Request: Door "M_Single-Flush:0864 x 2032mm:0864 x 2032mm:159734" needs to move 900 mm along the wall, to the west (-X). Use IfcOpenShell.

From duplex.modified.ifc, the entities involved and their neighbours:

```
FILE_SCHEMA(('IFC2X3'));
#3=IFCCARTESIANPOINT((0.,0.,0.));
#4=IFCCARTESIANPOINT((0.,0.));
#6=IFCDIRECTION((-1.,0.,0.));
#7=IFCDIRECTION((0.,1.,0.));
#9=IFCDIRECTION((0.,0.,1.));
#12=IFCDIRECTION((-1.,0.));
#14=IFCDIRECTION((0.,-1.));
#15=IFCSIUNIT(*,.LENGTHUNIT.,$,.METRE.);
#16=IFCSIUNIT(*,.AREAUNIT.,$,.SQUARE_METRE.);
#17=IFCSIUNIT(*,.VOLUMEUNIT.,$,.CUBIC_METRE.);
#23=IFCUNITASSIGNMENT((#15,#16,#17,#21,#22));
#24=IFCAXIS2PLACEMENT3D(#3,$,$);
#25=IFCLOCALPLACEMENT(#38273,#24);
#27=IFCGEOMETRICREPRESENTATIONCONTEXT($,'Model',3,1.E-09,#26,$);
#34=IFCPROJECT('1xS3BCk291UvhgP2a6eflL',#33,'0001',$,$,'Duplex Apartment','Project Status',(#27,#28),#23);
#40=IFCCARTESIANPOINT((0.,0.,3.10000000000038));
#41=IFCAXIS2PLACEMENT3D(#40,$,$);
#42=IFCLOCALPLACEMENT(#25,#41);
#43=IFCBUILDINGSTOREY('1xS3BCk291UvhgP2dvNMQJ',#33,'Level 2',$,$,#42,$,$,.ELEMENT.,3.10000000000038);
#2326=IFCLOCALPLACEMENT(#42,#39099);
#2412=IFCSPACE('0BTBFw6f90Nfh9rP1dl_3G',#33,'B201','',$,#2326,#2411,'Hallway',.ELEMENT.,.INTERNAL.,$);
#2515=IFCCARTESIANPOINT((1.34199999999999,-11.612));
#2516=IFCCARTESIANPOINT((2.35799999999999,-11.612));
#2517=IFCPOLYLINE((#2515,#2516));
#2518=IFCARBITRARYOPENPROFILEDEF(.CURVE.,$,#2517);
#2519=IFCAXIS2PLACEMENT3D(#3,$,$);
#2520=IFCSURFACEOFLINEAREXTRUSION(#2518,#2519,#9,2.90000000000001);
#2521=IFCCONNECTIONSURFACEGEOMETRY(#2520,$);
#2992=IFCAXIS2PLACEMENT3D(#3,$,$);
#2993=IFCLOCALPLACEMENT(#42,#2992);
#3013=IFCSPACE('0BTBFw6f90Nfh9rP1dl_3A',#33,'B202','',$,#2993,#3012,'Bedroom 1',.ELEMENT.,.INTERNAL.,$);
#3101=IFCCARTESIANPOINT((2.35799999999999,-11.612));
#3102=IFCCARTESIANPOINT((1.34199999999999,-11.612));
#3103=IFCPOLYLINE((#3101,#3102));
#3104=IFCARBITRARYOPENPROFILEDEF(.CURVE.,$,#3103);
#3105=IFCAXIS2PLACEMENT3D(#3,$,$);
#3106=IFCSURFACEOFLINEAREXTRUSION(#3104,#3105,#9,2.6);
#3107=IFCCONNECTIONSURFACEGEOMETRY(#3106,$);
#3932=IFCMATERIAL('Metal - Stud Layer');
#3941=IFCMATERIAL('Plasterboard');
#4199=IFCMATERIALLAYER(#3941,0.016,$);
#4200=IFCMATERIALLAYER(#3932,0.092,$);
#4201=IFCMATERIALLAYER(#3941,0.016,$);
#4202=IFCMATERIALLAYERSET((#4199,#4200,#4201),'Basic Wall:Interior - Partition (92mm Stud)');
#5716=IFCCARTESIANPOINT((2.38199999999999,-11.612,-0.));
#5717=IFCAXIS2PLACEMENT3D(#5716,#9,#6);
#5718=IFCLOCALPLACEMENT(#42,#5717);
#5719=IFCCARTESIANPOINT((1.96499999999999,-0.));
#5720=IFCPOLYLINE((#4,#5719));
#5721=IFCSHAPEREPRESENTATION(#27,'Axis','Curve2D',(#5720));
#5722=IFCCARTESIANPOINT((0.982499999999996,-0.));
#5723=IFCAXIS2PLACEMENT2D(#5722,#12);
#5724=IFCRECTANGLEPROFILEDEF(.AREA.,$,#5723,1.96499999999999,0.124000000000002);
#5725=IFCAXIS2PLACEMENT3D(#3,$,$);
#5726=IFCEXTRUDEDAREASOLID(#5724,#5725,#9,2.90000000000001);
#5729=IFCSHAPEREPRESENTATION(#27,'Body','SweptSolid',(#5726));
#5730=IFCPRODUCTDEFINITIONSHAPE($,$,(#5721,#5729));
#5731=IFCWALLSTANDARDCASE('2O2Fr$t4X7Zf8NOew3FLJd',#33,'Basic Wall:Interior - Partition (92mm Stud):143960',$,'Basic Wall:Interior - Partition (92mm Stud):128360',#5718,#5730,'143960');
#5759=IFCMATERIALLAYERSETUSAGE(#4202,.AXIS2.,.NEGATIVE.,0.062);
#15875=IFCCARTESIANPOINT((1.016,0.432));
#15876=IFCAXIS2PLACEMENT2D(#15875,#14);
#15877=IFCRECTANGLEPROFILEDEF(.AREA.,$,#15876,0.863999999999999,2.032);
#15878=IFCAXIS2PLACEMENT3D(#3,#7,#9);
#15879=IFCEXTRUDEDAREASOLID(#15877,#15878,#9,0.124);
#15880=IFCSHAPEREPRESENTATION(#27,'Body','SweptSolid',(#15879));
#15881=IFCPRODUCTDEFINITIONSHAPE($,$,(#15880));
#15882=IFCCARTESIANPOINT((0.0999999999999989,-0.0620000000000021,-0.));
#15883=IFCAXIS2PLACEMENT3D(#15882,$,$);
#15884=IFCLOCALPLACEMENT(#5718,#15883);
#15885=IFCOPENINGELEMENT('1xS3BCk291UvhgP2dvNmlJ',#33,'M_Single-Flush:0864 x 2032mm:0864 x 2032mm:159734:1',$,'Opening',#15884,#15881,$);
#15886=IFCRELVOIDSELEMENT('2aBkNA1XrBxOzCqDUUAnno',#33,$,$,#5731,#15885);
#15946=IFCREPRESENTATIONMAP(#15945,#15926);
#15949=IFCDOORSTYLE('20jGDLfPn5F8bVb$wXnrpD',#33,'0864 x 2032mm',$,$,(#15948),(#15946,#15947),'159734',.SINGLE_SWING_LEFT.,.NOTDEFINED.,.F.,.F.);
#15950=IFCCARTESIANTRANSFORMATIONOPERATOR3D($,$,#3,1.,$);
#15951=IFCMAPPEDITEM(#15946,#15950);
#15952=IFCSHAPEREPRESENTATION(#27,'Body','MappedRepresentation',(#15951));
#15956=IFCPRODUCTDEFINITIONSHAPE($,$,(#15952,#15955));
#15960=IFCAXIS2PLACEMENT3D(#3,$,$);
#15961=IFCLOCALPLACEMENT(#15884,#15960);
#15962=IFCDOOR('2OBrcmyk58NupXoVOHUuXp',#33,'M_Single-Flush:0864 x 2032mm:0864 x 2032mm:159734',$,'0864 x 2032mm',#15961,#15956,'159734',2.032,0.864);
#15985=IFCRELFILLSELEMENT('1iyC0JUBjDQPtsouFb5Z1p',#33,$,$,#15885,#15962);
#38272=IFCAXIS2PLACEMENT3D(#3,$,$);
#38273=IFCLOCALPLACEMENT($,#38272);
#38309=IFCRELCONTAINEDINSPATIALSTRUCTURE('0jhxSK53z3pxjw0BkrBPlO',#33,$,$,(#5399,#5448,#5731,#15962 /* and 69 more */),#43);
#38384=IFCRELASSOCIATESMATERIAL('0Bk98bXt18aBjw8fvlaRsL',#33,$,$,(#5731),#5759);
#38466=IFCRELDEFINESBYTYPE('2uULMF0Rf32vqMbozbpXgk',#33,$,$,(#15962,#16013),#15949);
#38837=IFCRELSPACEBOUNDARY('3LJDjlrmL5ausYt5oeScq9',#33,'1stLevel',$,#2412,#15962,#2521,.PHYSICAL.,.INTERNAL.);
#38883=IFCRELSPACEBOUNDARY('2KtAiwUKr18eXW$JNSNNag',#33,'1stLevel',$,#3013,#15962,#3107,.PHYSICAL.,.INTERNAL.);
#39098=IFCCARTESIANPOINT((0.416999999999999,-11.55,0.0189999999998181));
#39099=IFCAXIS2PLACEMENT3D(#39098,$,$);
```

```python
import numpy as np
import ifcopenshell
import ifcopenshell.api.geometry
import ifcopenshell.util.placement
import ifcopenshell.util.unit

model = ifcopenshell.open("duplex.modified.ifc")
unit_scale = ifcopenshell.util.unit.calculate_unit_scale(model)

door = model.by_guid("2OBrcmyk58NupXoVOHUuXp")
opening = door.FillsVoids[0].RelatingOpeningElement
wall = opening.VoidsElements[0].RelatingBuildingElement

wall_matrix = ifcopenshell.util.placement.get_local_placement(wall.ObjectPlacement)
shift = wall_matrix[:3, 0] * 0.9 / unit_scale
before = ifcopenshell.util.placement.get_local_placement(door.ObjectPlacement)[:3, 3].copy()

# The door is placed relative to its opening, so it follows when the opening moves.
matrix = ifcopenshell.util.placement.get_local_placement(opening.ObjectPlacement)
matrix[:3, 3] += shift
ifcopenshell.api.geometry.edit_object_placement(
    model, product=opening, matrix=matrix, is_si=False, should_transform_children=True
)

# Space boundary surfaces are stored in each space's coordinates; move them too.
for rel in door.ProvidesBoundaries:
    if not rel.ConnectionGeometry:
        continue
    surface = rel.ConnectionGeometry.SurfaceOnRelatingElement
    space_matrix = ifcopenshell.util.placement.get_local_placement(rel.RelatingSpace.ObjectPlacement)
    point = np.array(surface.Position.Location.Coordinates) + space_matrix[:3, :3].T @ shift
    surface.Position = model.createIfcAxis2Placement3D(
        model.createIfcCartesianPoint(point.tolist()), surface.Position.Axis, surface.Position.RefDirection
    )

after = ifcopenshell.util.placement.get_local_placement(door.ObjectPlacement)[:3, 3]
print("door moved by", (after - before).round(3) + 0.0)

model.write("duplex.modified_v2.ifc")
```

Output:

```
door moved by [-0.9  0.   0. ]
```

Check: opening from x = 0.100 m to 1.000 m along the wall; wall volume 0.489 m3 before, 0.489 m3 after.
